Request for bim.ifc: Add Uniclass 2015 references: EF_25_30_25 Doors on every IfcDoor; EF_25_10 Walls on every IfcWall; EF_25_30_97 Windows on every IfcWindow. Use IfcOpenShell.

First a look at what the model holds.

```python
import ifcopenshell

model = ifcopenshell.open("bim.ifc")
print(model.schema)
print("classifications:", [c.Name for c in model.by_type("IfcClassification")])
for ifc_class in ("IfcDoor", "IfcRoof", "IfcStair", "IfcWall", "IfcWindow"):
    print(ifc_class, len(model.by_type(ifc_class)))
```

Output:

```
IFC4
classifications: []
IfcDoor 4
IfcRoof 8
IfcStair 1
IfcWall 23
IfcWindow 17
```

```python
import ifcopenshell
import ifcopenshell.api.classification

model = ifcopenshell.open("bim.ifc")

system = ifcopenshell.api.classification.add_classification(model, classification="Uniclass 2015")

codes = {
    "IfcDoor": ("EF_25_30_25", "Doors"),
    "IfcWall": ("EF_25_10", "Walls"),
    "IfcWindow": ("EF_25_30_97", "Windows"),
}
for ifc_class, (code, name) in codes.items():
    products = model.by_type(ifc_class)
    ifcopenshell.api.classification.add_reference(
        model, products=products, classification=system, identification=code, name=name
    )
    print(code, len(products))

model.write("bim_rev.ifc")
```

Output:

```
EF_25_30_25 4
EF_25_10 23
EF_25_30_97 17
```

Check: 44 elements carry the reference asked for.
